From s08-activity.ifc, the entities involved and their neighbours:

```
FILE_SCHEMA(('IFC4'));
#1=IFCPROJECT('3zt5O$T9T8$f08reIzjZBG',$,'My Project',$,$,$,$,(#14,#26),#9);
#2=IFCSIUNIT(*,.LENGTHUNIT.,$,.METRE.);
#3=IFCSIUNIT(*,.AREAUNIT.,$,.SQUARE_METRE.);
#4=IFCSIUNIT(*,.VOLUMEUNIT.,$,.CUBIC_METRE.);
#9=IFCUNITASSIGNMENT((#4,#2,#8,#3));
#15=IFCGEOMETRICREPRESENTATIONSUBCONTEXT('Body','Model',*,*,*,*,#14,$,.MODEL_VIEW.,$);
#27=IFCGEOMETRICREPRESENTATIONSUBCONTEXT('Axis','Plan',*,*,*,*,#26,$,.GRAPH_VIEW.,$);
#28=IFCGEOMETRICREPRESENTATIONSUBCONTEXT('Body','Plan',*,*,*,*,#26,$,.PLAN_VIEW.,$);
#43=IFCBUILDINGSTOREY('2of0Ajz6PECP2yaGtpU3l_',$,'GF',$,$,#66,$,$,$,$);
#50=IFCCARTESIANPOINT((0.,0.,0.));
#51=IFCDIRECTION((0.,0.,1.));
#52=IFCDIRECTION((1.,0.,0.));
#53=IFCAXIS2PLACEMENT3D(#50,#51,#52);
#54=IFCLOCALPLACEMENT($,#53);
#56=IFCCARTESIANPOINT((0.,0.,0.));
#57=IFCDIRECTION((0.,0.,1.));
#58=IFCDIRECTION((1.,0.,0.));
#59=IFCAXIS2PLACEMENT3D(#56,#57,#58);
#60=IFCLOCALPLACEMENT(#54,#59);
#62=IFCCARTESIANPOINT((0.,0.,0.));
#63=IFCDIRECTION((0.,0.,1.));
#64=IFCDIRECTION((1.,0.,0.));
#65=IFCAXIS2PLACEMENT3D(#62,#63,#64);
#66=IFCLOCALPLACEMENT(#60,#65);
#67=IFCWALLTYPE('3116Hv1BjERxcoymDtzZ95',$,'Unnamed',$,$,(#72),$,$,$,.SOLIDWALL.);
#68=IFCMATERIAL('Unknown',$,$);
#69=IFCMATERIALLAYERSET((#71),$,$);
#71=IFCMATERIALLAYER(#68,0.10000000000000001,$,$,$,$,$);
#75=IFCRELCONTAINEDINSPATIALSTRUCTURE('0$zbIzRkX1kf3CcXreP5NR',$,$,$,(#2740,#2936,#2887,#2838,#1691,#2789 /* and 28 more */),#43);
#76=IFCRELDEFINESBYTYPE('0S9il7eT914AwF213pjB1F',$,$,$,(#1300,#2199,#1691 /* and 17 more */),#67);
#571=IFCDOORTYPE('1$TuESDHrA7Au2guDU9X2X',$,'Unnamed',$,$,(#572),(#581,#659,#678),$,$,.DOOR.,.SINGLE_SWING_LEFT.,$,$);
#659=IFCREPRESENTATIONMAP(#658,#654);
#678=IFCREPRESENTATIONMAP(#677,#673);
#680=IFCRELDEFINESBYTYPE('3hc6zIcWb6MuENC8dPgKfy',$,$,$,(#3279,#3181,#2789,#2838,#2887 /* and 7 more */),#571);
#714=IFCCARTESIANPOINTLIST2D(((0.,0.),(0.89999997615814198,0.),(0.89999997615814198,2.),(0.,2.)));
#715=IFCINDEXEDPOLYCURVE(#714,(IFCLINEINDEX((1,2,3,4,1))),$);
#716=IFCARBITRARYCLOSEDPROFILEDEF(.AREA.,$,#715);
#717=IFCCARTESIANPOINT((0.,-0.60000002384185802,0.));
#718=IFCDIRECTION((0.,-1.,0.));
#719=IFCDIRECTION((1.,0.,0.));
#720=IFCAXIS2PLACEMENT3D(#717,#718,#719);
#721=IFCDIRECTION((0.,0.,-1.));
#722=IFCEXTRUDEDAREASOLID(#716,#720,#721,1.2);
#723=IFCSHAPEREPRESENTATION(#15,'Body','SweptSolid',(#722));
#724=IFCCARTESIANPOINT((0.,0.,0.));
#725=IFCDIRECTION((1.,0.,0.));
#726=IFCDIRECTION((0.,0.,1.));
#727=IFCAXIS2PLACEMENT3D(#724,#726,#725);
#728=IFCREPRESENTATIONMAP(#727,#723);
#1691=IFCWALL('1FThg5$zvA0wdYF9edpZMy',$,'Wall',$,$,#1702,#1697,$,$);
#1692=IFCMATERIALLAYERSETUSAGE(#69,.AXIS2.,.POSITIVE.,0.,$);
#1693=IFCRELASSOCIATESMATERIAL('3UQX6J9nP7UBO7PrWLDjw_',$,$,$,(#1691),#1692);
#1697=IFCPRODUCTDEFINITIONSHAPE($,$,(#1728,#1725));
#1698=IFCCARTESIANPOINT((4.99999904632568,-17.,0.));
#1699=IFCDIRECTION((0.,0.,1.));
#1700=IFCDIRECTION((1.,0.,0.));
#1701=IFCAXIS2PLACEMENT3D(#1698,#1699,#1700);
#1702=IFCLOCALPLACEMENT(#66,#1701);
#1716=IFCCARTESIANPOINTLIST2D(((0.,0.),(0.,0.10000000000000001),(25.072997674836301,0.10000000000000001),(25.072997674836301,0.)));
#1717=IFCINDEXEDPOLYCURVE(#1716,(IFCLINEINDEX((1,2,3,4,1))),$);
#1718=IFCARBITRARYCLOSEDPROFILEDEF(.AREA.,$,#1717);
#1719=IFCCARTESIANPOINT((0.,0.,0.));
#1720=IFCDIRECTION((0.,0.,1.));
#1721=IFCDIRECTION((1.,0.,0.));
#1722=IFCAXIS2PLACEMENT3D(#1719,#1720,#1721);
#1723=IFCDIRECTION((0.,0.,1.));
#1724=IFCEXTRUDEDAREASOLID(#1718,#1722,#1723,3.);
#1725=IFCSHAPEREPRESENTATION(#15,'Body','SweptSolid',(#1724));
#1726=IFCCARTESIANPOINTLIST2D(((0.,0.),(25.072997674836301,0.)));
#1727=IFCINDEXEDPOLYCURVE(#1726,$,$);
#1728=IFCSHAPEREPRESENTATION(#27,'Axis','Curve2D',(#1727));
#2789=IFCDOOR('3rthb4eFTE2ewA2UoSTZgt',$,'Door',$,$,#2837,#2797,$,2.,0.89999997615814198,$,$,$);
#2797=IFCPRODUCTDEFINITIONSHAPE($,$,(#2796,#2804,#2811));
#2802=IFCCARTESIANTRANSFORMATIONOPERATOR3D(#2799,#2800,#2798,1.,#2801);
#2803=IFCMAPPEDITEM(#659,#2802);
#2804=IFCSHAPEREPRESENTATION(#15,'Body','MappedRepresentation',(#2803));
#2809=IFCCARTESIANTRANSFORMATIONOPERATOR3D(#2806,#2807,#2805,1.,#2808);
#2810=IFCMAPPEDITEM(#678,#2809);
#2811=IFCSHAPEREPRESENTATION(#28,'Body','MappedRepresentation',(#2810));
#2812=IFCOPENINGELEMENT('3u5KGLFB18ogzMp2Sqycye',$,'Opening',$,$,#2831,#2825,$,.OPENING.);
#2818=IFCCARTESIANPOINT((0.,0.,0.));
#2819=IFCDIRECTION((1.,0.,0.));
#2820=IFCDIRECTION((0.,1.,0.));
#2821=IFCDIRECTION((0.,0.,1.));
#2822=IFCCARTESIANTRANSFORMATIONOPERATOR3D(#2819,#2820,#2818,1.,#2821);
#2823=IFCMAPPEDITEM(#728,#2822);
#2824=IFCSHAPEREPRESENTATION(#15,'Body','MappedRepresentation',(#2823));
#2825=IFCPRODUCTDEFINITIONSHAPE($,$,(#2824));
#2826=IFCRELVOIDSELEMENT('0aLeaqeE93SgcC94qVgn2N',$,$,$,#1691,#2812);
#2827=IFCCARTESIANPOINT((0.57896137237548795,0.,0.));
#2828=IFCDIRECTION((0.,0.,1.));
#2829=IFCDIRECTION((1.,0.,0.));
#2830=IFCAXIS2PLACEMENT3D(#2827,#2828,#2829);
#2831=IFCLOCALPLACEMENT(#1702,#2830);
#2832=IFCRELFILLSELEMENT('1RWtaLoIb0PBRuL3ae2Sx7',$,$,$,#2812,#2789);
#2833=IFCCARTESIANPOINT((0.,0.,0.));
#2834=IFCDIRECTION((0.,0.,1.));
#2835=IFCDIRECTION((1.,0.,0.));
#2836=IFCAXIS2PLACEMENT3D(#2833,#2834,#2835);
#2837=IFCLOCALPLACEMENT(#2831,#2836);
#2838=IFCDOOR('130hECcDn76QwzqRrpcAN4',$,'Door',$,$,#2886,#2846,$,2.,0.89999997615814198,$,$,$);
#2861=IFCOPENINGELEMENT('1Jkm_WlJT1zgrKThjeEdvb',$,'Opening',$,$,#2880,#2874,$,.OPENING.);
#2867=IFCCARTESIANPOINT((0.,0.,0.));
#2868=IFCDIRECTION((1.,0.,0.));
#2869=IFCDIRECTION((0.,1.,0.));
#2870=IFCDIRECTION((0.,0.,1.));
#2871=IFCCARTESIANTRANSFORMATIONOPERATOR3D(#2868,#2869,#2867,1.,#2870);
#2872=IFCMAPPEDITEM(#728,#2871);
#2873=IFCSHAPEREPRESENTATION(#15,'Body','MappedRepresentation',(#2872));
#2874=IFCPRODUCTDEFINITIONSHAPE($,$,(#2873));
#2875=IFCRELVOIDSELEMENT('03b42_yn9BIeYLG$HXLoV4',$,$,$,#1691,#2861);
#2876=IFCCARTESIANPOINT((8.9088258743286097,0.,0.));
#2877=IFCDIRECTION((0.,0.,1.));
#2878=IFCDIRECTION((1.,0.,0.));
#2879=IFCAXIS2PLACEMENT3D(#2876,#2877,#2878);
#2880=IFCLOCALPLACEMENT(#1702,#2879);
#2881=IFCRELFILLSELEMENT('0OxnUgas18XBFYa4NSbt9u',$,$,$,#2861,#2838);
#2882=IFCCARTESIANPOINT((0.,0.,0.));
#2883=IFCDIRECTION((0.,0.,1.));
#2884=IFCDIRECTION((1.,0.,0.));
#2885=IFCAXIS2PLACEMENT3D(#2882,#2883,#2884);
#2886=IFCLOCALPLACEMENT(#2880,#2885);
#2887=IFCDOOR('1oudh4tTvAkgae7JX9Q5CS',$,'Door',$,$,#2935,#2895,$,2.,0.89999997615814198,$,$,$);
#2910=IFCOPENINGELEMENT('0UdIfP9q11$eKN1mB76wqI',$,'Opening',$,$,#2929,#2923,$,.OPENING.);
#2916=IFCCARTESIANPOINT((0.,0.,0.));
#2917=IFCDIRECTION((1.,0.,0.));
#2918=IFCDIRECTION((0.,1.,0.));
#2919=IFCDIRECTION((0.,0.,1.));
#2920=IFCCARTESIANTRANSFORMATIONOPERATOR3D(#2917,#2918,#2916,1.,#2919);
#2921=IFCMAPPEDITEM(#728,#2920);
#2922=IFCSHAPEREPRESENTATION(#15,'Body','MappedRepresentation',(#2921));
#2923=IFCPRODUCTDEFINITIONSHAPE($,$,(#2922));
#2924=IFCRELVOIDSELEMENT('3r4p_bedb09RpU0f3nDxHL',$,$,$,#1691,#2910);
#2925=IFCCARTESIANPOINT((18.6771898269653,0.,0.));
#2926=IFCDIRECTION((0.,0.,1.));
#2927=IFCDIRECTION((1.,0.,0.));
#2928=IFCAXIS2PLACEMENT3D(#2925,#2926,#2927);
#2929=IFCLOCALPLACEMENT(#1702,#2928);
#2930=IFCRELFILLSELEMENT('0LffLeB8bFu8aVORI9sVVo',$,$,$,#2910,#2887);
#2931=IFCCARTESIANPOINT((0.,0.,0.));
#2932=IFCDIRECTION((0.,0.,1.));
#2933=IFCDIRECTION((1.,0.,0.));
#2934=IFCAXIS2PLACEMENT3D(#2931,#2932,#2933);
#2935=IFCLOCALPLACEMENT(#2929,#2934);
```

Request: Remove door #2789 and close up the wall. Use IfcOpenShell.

```python
import ifcopenshell
import ifcopenshell.api.feature
import ifcopenshell.api.root
import ifcopenshell.geom
import ifcopenshell.util.shape

model = ifcopenshell.open("s08-activity.ifc")
settings = ifcopenshell.geom.settings()


def volume(element):
    """Net volume in cubic metres, openings subtracted."""
    shape = ifcopenshell.geom.create_shape(settings, element)
    return ifcopenshell.util.shape.get_volume(shape.geometry)


door = model.by_guid("3rthb4eFTE2ewA2UoSTZgt")
opening = door.FillsVoids[0].RelatingOpeningElement
wall = opening.VoidsElements[0].RelatingBuildingElement
before = volume(wall)

ifcopenshell.api.root.remove_product(model, product=door)
ifcopenshell.api.feature.remove_feature(model, feature=opening)

after = volume(wall)

print(f"wall volume {before:.3f} -> {after:.3f} m3")

model.write("s08-activity_v2.ifc")
```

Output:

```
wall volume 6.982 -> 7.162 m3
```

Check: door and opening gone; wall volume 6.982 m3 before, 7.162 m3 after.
